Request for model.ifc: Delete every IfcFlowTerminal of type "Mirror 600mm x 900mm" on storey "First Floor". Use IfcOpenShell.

First a look at what the model holds.

```python
import ifcopenshell
import ifcopenshell.util.element

model = ifcopenshell.open("model.ifc")
print(model.schema)
storey = next(s for s in model.by_type("IfcBuildingStorey") if s.Name == "First Floor")
terminals = [e for e in ifcopenshell.util.element.get_decomposition(storey) if e.is_a("IfcFlowTerminal")]
seen = {}
for e in terminals:
    element_type = ifcopenshell.util.element.get_type(e)
    name = element_type.Name if element_type not in (None, e) else None
    seen[name] = seen.get(name, 0) + 1
for name, count in sorted(seen.items(), key=str):
    print(count, "x", name)
```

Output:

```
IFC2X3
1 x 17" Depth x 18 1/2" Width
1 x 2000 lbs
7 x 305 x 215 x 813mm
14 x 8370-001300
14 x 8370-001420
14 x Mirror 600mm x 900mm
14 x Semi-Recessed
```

```python
import ifcopenshell
import ifcopenshell.api.root
import ifcopenshell.util.element

model = ifcopenshell.open("model.ifc")

storey = next(s for s in model.by_type("IfcBuildingStorey") if s.Name == "First Floor")
terminals = [e for e in ifcopenshell.util.element.get_decomposition(storey) if e.is_a("IfcFlowTerminal")]
targets = [e for e in terminals if (t := ifcopenshell.util.element.get_type(e)) not in (None, e) and t.Name == "Mirror 600mm x 900mm"]

for e in targets:
    ifcopenshell.api.root.remove_product(model, product=e)
print(len(targets), "removed")

model.write("model_rev.ifc")
```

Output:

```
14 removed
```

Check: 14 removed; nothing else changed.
